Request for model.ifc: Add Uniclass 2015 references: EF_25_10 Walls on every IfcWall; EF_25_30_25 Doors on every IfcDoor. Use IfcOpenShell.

First a look at what the model holds.

```python
import ifcopenshell

model = ifcopenshell.open("model.ifc")
print(model.schema)
print("classifications:", [c.Name for c in model.by_type("IfcClassification")])
for ifc_class in ("IfcDoor", "IfcRoof", "IfcStair", "IfcWall", "IfcWindow"):
    print(ifc_class, len(model.by_type(ifc_class)))
```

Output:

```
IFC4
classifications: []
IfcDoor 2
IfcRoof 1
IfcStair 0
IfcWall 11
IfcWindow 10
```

```python
import ifcopenshell
import ifcopenshell.api.classification

model = ifcopenshell.open("model.ifc")

system = ifcopenshell.api.classification.add_classification(model, classification="Uniclass 2015")

codes = {
    "IfcWall": ("EF_25_10", "Walls"),
    "IfcDoor": ("EF_25_30_25", "Doors"),
}
for ifc_class, (code, name) in codes.items():
    products = model.by_type(ifc_class)
    ifcopenshell.api.classification.add_reference(
        model, products=products, classification=system, identification=code, name=name
    )
    print(code, len(products))

model.write("model_rev.ifc")
```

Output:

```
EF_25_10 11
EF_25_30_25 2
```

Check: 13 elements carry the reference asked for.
